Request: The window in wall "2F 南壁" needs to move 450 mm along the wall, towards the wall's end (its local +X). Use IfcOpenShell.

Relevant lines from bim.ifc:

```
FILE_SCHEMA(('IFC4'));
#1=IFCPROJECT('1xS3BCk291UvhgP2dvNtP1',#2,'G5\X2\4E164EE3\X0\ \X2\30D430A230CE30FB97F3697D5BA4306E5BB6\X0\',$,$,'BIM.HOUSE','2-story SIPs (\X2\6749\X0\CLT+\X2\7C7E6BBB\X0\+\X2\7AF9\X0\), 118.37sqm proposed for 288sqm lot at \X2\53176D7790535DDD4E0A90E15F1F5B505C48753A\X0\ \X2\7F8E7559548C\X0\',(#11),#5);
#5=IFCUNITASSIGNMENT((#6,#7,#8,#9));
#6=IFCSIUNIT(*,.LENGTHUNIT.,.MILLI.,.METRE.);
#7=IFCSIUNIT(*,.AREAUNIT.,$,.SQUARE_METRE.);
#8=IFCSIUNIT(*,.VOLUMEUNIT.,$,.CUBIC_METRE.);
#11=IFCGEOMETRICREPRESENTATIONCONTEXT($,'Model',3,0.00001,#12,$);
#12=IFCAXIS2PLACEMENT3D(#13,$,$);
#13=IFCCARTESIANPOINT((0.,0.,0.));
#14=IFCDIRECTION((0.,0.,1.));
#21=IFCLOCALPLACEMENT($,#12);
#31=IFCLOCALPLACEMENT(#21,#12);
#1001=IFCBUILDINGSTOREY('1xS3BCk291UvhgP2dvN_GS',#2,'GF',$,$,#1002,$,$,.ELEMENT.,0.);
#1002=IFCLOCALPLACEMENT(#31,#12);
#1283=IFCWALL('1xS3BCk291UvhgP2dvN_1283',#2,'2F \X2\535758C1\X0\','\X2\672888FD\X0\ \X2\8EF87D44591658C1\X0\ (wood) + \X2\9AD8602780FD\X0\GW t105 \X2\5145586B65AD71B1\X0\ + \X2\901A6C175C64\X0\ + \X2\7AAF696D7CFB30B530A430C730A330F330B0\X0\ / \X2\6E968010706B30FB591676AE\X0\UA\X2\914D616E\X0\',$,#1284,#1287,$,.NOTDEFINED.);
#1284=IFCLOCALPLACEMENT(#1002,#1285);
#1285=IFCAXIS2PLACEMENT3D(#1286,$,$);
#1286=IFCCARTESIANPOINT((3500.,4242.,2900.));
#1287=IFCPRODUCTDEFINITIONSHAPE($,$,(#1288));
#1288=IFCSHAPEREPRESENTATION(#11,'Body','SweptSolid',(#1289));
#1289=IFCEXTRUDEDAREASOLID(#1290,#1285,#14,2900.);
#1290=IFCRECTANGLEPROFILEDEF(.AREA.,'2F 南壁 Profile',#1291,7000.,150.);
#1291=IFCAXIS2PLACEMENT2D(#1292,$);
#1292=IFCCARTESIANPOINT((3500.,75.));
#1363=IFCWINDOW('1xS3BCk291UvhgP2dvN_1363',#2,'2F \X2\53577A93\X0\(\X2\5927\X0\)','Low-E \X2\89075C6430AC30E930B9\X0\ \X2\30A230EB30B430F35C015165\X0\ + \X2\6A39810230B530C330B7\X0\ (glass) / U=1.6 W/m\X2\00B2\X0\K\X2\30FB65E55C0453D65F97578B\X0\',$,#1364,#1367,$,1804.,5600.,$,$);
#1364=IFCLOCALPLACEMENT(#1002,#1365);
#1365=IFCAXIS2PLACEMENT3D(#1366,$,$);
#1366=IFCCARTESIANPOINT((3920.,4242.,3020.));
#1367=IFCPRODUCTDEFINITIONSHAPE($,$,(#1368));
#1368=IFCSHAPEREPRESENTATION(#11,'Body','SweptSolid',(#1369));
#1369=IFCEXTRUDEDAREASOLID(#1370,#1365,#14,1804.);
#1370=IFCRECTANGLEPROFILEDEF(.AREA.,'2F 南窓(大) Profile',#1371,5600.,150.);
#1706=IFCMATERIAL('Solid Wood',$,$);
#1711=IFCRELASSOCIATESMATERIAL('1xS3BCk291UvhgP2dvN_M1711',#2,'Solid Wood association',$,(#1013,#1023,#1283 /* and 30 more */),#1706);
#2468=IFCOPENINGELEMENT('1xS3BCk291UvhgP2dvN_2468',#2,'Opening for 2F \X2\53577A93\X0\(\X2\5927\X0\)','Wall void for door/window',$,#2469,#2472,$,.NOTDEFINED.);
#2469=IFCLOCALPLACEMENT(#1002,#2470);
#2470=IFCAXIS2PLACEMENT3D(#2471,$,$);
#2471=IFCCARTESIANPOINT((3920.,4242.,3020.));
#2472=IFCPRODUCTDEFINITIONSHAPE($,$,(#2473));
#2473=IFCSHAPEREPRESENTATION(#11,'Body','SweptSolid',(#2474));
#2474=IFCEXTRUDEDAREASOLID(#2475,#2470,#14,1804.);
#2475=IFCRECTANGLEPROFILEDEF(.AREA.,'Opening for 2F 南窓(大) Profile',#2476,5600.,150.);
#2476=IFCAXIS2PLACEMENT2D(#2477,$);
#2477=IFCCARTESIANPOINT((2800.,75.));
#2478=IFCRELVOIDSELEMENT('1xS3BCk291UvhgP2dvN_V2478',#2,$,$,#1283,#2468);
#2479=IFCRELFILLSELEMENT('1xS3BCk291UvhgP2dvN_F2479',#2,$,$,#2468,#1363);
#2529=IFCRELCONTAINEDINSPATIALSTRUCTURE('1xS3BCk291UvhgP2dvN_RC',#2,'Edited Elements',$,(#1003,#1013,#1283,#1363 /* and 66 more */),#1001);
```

```python
import ifcopenshell
import ifcopenshell.api.geometry
import ifcopenshell.util.placement
import ifcopenshell.util.unit

model = ifcopenshell.open("bim.ifc")
unit_scale = ifcopenshell.util.unit.calculate_unit_scale(model)

window = model.by_guid("1xS3BCk291UvhgP2dvN_1363")
opening = window.FillsVoids[0].RelatingOpeningElement
wall = opening.VoidsElements[0].RelatingBuildingElement

wall_matrix = ifcopenshell.util.placement.get_local_placement(wall.ObjectPlacement)
shift = wall_matrix[:3, 0] * 0.45 / unit_scale
before = ifcopenshell.util.placement.get_local_placement(window.ObjectPlacement)[:3, 3].copy()

# The window is not placed relative to its opening, so move both.
for product in (opening, window):
    matrix = ifcopenshell.util.placement.get_local_placement(product.ObjectPlacement)
    matrix[:3, 3] += shift
    ifcopenshell.api.geometry.edit_object_placement(model, product=product, matrix=matrix, is_si=False)

after = ifcopenshell.util.placement.get_local_placement(window.ObjectPlacement)[:3, 3]
print("window moved by", (after - before).round(3) + 0.0)

model.write("bim_edited.ifc")
```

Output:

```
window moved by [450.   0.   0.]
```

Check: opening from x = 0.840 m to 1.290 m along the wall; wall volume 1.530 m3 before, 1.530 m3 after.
